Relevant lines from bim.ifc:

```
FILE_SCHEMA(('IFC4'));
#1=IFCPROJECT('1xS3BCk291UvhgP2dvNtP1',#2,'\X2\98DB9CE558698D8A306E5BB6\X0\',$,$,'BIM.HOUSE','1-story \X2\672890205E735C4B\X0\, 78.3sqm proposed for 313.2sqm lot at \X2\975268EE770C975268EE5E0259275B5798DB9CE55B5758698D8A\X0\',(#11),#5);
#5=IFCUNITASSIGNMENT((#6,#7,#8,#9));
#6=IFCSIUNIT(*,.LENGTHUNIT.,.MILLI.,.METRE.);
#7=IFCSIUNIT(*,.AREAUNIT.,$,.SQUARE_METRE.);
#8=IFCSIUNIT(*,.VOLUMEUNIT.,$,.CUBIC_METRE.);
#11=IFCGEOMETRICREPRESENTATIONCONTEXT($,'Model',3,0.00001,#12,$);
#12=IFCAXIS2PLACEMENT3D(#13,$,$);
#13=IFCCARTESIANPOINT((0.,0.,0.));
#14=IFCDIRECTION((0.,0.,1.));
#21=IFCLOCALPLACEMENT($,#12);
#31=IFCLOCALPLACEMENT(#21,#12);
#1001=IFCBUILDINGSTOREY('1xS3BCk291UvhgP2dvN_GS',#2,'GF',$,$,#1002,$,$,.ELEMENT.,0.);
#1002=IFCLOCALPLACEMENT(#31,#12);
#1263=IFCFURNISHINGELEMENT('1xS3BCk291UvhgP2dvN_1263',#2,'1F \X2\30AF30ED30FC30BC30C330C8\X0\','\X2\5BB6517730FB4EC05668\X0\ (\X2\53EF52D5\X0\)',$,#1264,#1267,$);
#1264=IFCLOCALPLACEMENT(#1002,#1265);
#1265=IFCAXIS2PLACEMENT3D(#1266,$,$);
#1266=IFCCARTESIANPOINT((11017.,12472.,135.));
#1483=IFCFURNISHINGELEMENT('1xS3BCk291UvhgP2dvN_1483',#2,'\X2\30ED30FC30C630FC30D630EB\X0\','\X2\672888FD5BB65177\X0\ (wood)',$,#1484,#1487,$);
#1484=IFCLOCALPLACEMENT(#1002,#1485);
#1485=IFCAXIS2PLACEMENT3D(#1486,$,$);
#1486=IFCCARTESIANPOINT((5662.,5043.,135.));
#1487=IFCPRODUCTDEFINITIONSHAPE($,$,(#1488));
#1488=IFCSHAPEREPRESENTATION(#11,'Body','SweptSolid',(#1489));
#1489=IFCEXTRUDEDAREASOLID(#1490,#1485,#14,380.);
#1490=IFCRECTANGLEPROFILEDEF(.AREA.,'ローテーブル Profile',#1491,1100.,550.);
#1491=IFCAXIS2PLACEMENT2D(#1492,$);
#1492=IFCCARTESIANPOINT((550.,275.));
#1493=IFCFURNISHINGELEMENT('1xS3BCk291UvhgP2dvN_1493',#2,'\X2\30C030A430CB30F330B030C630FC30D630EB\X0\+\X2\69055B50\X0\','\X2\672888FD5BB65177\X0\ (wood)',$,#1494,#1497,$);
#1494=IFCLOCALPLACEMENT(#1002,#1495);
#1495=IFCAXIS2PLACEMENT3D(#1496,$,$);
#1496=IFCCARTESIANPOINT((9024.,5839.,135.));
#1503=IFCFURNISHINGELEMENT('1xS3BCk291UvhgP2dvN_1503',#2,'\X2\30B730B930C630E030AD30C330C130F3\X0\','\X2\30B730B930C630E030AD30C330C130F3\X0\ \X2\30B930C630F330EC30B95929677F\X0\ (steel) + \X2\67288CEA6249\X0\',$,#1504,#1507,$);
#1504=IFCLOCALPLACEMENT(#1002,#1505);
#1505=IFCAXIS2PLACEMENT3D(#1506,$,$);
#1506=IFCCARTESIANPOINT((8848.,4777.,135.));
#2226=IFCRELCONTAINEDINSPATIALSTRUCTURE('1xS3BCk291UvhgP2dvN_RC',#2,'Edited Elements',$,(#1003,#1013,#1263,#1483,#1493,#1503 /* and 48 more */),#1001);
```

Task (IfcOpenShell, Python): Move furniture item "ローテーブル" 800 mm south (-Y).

```python
import ifcopenshell
import ifcopenshell.api.geometry
import ifcopenshell.util.placement
import ifcopenshell.util.unit

model = ifcopenshell.open("bim.ifc")
unit_scale = ifcopenshell.util.unit.calculate_unit_scale(model)

item = model.by_guid("1xS3BCk291UvhgP2dvN_1483")
matrix = ifcopenshell.util.placement.get_local_placement(item.ObjectPlacement)
matrix[1, 3] -= 0.8 / unit_scale
ifcopenshell.api.geometry.edit_object_placement(model, product=item, matrix=matrix, is_si=False)

print(ifcopenshell.util.placement.get_local_placement(item.ObjectPlacement).round(3) + 0.0)

model.write("bim_edited.ifc")
```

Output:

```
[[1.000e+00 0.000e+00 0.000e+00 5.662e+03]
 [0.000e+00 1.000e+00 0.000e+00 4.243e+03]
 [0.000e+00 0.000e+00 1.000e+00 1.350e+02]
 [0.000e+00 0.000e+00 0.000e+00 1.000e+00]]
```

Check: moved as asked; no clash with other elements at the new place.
